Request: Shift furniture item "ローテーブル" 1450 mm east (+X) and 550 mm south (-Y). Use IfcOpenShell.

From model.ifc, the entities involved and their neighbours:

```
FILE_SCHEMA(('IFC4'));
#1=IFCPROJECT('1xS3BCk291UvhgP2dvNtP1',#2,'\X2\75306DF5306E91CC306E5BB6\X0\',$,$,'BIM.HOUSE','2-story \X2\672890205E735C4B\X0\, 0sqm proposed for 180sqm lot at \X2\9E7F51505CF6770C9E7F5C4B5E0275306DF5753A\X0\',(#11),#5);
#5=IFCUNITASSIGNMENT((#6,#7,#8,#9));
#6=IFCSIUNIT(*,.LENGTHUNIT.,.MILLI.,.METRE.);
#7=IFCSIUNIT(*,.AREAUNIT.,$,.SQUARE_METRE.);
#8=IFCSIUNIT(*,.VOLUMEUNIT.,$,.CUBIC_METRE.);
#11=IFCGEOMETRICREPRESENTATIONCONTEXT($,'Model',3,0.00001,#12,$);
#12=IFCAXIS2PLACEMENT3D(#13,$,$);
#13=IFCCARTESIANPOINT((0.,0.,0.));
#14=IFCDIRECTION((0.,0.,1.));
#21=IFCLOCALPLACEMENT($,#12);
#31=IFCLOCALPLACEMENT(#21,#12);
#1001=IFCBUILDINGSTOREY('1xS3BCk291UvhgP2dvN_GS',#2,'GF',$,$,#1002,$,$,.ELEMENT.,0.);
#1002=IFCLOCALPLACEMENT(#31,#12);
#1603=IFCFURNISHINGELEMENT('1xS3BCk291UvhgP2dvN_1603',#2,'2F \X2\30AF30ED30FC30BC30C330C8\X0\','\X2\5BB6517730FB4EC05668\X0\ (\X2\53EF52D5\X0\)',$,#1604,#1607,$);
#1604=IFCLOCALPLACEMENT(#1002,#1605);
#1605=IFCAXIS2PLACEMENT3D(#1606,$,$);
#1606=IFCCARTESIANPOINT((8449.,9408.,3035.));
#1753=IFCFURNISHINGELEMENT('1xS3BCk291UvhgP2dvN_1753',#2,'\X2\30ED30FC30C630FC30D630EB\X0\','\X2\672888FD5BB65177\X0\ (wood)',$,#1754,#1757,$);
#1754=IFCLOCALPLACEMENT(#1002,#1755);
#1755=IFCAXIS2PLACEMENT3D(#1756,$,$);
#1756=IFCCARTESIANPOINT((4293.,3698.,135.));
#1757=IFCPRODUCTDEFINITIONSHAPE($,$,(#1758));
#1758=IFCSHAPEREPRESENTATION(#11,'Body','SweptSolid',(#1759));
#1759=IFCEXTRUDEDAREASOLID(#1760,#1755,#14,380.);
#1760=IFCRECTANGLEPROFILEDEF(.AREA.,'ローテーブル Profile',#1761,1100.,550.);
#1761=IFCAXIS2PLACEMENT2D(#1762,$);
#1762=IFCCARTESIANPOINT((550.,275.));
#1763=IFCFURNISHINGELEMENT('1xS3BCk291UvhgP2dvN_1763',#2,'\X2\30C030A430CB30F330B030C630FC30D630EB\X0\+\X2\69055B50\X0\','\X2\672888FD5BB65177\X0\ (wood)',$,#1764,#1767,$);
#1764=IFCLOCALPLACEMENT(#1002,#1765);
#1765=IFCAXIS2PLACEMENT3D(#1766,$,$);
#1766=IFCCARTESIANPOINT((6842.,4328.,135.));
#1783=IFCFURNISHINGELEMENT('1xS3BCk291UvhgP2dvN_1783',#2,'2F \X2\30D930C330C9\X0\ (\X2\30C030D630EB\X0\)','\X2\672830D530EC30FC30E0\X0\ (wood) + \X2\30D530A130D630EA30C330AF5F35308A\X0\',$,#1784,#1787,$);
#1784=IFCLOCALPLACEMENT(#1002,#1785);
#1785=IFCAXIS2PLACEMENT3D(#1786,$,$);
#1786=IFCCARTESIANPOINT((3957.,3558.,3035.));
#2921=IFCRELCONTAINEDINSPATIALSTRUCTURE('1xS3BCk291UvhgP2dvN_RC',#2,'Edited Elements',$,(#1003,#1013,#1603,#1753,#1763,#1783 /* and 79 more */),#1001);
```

```python
import ifcopenshell
import ifcopenshell.api.geometry
import ifcopenshell.util.placement

model = ifcopenshell.open("model.ifc")

item = model.by_id(1753)
matrix = ifcopenshell.util.placement.get_local_placement(item.ObjectPlacement)
matrix[0, 3] += 1450.0
matrix[1, 3] -= 550.0
ifcopenshell.api.geometry.edit_object_placement(model, product=item, matrix=matrix, is_si=False)

print(ifcopenshell.util.placement.get_local_placement(item.ObjectPlacement).round(3) + 0.0)

model.write("model_v2.ifc")
```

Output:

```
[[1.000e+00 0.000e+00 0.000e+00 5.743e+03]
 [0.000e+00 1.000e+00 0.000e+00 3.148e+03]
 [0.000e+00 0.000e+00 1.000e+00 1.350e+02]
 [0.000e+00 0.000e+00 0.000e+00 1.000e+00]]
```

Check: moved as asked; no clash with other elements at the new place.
